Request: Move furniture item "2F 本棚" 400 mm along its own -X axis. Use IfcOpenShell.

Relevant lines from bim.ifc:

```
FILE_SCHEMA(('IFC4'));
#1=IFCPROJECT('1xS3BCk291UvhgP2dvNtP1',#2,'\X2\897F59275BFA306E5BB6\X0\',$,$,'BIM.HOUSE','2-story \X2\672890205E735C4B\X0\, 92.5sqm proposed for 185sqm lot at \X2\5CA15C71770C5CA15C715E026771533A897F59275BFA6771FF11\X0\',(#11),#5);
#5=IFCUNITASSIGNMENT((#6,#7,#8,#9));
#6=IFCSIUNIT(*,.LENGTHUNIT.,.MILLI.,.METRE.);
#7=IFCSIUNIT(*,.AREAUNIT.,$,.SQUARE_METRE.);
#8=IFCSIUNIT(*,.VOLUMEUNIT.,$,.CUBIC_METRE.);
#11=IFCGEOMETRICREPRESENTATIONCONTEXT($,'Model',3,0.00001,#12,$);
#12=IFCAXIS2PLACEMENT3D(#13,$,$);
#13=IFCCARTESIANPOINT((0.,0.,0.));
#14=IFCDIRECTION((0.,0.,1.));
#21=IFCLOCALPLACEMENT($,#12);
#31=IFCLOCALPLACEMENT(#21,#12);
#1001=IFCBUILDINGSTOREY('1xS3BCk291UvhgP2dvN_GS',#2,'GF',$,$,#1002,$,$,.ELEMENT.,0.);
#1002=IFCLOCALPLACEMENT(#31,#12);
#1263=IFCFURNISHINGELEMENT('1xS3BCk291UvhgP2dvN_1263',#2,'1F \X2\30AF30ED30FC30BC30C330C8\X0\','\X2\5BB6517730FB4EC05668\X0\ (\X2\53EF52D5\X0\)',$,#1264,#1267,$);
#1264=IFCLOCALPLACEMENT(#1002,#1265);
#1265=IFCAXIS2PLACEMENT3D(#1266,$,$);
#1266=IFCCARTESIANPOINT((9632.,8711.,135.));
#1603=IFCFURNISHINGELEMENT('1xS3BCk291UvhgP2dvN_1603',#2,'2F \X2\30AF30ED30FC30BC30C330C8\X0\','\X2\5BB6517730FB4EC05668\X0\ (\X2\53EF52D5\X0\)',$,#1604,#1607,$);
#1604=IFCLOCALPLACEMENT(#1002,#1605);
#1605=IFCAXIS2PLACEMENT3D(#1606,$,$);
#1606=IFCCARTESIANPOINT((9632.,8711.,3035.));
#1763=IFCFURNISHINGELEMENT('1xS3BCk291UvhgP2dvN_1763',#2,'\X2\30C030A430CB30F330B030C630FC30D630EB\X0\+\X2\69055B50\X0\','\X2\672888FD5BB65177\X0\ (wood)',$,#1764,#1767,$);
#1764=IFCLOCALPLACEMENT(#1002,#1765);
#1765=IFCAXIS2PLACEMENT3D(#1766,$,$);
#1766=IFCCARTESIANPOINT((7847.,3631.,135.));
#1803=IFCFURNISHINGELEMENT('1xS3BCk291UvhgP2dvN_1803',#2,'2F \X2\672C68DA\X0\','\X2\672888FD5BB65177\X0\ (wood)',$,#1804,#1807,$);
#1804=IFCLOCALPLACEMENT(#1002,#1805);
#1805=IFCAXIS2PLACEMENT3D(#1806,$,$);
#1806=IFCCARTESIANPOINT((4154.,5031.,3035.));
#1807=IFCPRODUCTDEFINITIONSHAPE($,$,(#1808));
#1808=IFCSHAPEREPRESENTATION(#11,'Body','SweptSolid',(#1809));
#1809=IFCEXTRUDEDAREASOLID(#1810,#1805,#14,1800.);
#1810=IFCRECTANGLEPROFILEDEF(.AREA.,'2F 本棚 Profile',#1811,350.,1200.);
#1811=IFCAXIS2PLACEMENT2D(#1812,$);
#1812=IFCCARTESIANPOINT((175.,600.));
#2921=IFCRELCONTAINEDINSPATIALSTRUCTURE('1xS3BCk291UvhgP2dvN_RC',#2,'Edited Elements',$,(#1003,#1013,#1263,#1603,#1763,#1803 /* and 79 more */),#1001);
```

```python
import ifcopenshell
import ifcopenshell.api.geometry
import ifcopenshell.util.placement
import ifcopenshell.util.unit

model = ifcopenshell.open("bim.ifc")
unit_scale = ifcopenshell.util.unit.calculate_unit_scale(model)

item = model.by_guid("1xS3BCk291UvhgP2dvN_1803")
matrix = ifcopenshell.util.placement.get_local_placement(item.ObjectPlacement)
matrix[:3, 3] -= matrix[:3, 0] * 0.4 / unit_scale
ifcopenshell.api.geometry.edit_object_placement(model, product=item, matrix=matrix, is_si=False)

print(ifcopenshell.util.placement.get_local_placement(item.ObjectPlacement).round(3) + 0.0)

model.write("bim_v2.ifc")
```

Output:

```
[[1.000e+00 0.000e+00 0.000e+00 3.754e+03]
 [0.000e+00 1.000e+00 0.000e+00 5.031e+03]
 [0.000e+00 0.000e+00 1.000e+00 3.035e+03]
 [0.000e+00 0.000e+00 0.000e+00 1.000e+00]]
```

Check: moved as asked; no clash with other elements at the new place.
